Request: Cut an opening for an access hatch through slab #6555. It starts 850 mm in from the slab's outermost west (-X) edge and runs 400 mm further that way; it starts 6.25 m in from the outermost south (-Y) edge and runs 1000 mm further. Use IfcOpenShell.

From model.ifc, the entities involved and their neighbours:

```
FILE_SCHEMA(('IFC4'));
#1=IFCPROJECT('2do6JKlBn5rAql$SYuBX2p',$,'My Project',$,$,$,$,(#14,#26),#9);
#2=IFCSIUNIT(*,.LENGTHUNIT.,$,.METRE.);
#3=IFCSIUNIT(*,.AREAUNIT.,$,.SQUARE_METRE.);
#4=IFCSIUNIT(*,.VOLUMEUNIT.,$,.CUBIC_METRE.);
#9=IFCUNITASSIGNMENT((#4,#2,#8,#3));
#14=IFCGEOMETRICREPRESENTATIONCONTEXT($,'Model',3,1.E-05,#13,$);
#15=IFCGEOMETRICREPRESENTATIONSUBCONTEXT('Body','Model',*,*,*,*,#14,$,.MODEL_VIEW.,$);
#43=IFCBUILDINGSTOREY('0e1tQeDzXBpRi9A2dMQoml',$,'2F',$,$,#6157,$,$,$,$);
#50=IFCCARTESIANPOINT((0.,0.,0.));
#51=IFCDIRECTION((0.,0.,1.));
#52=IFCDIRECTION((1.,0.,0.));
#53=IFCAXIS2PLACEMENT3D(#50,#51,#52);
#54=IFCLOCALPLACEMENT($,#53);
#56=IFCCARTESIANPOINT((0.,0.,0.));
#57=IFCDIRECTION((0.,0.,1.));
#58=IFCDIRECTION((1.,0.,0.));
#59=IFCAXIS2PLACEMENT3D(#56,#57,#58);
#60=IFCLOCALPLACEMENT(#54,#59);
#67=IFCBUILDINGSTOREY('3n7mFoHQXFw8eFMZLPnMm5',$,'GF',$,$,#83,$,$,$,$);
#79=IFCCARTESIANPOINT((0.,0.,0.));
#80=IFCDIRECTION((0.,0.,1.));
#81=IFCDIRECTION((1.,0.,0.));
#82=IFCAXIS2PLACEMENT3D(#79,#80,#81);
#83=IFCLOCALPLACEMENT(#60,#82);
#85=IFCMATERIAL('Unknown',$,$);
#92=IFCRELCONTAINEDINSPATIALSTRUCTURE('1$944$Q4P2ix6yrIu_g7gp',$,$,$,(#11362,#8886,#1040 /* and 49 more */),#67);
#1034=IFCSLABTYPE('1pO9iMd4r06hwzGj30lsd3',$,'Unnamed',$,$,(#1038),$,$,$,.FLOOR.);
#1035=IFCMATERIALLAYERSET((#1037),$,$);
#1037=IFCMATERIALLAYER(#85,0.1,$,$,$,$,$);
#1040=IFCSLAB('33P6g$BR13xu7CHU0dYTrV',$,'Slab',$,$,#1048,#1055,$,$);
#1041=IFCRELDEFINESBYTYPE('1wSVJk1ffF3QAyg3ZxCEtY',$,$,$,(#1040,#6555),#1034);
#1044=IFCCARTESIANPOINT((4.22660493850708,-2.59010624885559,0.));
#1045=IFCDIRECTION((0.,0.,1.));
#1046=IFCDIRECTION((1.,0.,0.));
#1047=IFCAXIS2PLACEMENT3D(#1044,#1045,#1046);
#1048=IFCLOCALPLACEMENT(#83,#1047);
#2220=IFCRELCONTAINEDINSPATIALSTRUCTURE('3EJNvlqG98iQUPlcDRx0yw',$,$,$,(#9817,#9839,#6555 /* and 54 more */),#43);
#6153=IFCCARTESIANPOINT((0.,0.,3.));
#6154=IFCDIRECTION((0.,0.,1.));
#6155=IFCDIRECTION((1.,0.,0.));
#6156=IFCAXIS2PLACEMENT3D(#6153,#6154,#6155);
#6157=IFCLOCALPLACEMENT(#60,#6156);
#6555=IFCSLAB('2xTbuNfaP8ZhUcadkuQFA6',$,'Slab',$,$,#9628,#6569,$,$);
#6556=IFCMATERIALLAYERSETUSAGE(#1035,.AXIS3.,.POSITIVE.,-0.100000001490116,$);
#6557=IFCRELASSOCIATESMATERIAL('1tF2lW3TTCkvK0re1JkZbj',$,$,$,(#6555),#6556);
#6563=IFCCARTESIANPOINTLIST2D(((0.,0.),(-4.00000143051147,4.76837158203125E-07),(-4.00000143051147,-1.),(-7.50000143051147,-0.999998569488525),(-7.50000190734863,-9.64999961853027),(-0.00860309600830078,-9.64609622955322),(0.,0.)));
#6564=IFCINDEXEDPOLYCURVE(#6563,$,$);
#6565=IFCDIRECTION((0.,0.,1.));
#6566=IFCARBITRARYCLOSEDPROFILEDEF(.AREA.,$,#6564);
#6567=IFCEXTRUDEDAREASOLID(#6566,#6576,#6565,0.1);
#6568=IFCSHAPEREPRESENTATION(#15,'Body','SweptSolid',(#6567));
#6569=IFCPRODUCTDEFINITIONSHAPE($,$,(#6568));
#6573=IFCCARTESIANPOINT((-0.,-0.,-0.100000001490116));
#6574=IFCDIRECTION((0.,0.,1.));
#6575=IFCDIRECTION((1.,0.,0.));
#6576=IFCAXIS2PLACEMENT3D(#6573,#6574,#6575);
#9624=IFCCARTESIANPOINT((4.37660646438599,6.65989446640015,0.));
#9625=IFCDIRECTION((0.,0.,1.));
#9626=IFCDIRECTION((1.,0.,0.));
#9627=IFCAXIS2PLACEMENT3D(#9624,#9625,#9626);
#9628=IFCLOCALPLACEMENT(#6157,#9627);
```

```python
import numpy as np
import ifcopenshell
import ifcopenshell.api.feature
import ifcopenshell.api.geometry
import ifcopenshell.api.root
import ifcopenshell.geom
import ifcopenshell.util.placement
import ifcopenshell.util.representation
import ifcopenshell.util.shape
import ifcopenshell.util.unit

model = ifcopenshell.open("model.ifc")
unit_scale = ifcopenshell.util.unit.calculate_unit_scale(model)
settings = ifcopenshell.geom.settings()


def volume(element):
    """Net volume in cubic metres, openings subtracted."""
    shape = ifcopenshell.geom.create_shape(settings, element)
    return ifcopenshell.util.shape.get_volume(shape.geometry)


slab = model.by_guid("2xTbuNfaP8ZhUcadkuQFA6")
before = volume(slab)

# Extent in the slab's own axes, in metres. The edges named are its -X and -Y sides.
slab_shape = ifcopenshell.geom.create_shape(settings, slab)
vertices = ifcopenshell.util.shape.get_vertices(slab_shape.geometry)
x_min, y_min, bottom = vertices.min(axis=0)
top = vertices[:, 2].max()

opening = ifcopenshell.api.root.create_entity(model, ifc_class="IfcOpeningElement", name="Access hatch opening", predefined_type="OPENING")
context = ifcopenshell.util.representation.get_context(model, "Model", "Body", "MODEL_VIEW")
width, depth = 0.4, 1
outline = [(0.0, 0.0), (width, 0.0), (width, depth), (0.0, depth), (0.0, 0.0)]
# Overshoot both faces by 50 mm so the cut is clean.
shape = ifcopenshell.api.geometry.add_slab_representation(
    model, context=context, depth=top - bottom + 0.1, polyline=outline
)
ifcopenshell.api.geometry.assign_representation(model, product=opening, representation=shape)

matrix = ifcopenshell.util.placement.get_local_placement(slab.ObjectPlacement)
matrix[:, 3] = matrix @ np.append(np.array([x_min + 0.85, y_min + 6.25, bottom - 0.05]) / unit_scale, 1.0)
ifcopenshell.api.geometry.edit_object_placement(model, product=opening, matrix=matrix, is_si=False)
ifcopenshell.api.feature.add_feature(model, feature=opening, element=slab)

after = volume(slab)

print(f"slab volume {before:.3f} -> {after:.3f} m3")

model.write("model-out.ifc")
```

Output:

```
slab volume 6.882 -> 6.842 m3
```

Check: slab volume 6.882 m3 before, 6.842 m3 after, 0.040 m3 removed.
